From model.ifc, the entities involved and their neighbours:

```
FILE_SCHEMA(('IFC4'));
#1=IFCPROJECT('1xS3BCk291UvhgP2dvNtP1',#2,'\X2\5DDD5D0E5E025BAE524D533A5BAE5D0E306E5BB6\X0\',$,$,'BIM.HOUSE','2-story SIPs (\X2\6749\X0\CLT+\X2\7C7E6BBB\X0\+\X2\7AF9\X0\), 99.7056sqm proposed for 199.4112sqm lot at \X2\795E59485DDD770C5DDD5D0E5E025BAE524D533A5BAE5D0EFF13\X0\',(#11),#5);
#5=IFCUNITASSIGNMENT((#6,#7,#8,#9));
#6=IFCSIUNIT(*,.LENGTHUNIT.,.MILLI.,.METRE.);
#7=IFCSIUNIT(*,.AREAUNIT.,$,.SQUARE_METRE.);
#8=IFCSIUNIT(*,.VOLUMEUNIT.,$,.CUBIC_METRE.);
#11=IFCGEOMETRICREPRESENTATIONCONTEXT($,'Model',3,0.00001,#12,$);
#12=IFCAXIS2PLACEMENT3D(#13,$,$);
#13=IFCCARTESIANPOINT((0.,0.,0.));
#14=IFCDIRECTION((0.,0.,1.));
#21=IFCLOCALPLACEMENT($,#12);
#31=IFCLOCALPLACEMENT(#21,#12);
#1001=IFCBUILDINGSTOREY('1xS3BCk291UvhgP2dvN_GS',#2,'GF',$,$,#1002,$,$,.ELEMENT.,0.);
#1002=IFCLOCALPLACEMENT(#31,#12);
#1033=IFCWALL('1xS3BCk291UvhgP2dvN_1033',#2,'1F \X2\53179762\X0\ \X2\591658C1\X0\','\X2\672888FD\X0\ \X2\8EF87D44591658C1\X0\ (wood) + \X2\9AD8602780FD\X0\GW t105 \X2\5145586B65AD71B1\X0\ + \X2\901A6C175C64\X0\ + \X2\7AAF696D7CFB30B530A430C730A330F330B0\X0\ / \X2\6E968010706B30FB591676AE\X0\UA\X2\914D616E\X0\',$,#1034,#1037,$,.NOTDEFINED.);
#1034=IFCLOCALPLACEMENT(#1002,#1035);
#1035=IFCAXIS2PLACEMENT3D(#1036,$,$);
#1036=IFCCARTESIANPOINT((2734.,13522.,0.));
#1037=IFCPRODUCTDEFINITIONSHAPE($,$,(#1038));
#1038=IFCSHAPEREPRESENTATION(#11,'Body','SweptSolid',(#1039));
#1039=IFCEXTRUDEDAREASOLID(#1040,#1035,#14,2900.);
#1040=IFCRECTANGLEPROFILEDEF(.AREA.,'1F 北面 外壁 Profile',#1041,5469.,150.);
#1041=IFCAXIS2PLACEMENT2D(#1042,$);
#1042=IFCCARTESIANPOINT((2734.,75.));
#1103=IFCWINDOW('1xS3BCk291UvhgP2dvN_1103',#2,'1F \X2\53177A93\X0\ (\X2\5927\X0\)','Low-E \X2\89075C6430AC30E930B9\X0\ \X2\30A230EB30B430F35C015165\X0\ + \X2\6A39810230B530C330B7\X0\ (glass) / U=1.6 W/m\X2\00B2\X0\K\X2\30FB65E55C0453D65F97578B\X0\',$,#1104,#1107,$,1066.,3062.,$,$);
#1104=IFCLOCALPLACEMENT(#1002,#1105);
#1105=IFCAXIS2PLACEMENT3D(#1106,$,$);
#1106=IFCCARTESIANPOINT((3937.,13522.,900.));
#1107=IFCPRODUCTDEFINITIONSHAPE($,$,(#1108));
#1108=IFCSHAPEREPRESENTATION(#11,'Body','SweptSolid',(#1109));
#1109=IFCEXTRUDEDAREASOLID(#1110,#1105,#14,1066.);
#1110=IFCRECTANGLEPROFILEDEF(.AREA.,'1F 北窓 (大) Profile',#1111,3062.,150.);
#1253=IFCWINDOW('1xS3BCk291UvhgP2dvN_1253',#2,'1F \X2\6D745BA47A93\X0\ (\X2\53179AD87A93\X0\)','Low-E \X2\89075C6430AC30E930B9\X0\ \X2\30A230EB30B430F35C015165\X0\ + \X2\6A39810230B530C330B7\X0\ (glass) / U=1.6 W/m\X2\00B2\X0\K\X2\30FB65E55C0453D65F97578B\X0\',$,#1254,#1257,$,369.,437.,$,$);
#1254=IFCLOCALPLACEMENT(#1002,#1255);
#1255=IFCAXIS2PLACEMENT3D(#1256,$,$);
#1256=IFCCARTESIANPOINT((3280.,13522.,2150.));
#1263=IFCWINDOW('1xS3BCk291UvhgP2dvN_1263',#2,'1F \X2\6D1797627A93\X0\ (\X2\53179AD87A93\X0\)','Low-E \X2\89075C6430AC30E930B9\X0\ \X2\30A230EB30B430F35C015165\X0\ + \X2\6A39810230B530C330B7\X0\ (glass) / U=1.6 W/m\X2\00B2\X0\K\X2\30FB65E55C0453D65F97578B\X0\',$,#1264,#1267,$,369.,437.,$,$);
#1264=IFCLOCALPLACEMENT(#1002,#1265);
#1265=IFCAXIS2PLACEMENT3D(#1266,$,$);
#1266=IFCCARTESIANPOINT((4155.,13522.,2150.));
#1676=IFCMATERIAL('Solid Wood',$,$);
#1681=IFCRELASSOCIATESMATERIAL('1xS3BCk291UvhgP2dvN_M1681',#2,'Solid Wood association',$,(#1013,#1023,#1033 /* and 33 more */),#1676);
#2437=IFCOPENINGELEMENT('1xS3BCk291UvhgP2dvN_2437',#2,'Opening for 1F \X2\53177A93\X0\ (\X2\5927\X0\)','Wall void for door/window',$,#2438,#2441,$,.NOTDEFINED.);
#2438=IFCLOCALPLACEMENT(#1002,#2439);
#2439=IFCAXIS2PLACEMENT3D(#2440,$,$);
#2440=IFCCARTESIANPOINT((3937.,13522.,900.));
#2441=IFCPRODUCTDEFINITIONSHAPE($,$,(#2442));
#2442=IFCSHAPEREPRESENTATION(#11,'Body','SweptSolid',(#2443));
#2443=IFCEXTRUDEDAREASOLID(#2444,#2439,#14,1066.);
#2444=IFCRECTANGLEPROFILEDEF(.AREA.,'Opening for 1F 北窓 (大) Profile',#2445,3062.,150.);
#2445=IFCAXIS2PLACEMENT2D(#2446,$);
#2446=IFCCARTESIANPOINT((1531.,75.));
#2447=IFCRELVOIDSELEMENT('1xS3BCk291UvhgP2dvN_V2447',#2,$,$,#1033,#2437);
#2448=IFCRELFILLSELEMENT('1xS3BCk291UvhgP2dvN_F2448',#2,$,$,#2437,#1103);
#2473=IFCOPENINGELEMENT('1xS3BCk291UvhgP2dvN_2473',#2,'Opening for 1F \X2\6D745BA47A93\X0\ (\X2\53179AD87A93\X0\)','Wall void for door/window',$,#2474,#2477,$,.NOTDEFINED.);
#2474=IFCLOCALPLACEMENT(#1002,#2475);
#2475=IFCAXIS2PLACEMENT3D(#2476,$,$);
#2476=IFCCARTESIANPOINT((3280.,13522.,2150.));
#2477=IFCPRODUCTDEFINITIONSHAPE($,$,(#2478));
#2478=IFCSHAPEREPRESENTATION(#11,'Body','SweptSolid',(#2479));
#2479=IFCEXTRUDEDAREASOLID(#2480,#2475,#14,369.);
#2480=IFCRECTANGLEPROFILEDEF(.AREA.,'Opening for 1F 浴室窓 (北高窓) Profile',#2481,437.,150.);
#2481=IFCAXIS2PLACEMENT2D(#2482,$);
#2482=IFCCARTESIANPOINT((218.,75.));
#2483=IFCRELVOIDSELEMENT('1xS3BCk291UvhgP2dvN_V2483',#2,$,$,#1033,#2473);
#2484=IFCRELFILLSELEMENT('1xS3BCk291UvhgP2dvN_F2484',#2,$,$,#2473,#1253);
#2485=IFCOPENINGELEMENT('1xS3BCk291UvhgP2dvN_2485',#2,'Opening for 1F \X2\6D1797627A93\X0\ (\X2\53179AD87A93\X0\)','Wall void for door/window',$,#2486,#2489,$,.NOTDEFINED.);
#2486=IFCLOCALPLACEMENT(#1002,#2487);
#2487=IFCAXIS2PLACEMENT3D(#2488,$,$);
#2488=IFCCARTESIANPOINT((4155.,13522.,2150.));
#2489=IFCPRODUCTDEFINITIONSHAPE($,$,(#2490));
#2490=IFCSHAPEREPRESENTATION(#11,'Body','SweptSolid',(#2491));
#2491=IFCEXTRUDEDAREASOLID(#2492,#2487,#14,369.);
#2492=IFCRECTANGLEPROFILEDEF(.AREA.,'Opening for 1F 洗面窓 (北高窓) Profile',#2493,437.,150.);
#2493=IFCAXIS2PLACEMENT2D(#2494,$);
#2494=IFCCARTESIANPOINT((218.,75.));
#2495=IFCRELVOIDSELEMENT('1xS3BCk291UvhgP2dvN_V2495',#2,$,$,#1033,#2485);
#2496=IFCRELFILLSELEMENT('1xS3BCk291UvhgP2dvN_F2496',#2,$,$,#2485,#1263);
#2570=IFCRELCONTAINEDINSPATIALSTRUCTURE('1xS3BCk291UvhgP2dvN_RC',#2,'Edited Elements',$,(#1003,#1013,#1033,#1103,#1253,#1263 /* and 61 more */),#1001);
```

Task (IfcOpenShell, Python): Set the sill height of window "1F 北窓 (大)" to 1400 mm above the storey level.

```python
import numpy as np
import ifcopenshell
import ifcopenshell.api.geometry
import ifcopenshell.geom
import ifcopenshell.util.element
import ifcopenshell.util.placement
import ifcopenshell.util.shape
import ifcopenshell.util.unit

model = ifcopenshell.open("model.ifc")
unit_scale = ifcopenshell.util.unit.calculate_unit_scale(model)

window = model.by_guid("1xS3BCk291UvhgP2dvN_1103")
opening = window.FillsVoids[0].RelatingOpeningElement
storey = ifcopenshell.util.element.get_container(window, ifc_class="IfcBuildingStorey")
level = ifcopenshell.util.placement.get_local_placement(storey.ObjectPlacement)[2, 3]

# The opening's origin need not be at the sill, so measure its lowest point.
shape = ifcopenshell.geom.create_shape(ifcopenshell.geom.settings(), opening)
bottom = ifcopenshell.util.shape.get_shape_bottom_elevation(shape, shape.geometry) / unit_scale
dz = level + 1.4 / unit_scale - bottom

shift = np.array([0.0, 0.0, dz])
# The window is not placed relative to its opening, so move both.
for product in (opening, window):
    matrix = ifcopenshell.util.placement.get_local_placement(product.ObjectPlacement)
    matrix[:3, 3] += shift
    ifcopenshell.api.geometry.edit_object_placement(model, product=product, matrix=matrix, is_si=False)

print(f"moved by {dz * unit_scale:+.3f} m")

model.write("model_v2.ifc")
```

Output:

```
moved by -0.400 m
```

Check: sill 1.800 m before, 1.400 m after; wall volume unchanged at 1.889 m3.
